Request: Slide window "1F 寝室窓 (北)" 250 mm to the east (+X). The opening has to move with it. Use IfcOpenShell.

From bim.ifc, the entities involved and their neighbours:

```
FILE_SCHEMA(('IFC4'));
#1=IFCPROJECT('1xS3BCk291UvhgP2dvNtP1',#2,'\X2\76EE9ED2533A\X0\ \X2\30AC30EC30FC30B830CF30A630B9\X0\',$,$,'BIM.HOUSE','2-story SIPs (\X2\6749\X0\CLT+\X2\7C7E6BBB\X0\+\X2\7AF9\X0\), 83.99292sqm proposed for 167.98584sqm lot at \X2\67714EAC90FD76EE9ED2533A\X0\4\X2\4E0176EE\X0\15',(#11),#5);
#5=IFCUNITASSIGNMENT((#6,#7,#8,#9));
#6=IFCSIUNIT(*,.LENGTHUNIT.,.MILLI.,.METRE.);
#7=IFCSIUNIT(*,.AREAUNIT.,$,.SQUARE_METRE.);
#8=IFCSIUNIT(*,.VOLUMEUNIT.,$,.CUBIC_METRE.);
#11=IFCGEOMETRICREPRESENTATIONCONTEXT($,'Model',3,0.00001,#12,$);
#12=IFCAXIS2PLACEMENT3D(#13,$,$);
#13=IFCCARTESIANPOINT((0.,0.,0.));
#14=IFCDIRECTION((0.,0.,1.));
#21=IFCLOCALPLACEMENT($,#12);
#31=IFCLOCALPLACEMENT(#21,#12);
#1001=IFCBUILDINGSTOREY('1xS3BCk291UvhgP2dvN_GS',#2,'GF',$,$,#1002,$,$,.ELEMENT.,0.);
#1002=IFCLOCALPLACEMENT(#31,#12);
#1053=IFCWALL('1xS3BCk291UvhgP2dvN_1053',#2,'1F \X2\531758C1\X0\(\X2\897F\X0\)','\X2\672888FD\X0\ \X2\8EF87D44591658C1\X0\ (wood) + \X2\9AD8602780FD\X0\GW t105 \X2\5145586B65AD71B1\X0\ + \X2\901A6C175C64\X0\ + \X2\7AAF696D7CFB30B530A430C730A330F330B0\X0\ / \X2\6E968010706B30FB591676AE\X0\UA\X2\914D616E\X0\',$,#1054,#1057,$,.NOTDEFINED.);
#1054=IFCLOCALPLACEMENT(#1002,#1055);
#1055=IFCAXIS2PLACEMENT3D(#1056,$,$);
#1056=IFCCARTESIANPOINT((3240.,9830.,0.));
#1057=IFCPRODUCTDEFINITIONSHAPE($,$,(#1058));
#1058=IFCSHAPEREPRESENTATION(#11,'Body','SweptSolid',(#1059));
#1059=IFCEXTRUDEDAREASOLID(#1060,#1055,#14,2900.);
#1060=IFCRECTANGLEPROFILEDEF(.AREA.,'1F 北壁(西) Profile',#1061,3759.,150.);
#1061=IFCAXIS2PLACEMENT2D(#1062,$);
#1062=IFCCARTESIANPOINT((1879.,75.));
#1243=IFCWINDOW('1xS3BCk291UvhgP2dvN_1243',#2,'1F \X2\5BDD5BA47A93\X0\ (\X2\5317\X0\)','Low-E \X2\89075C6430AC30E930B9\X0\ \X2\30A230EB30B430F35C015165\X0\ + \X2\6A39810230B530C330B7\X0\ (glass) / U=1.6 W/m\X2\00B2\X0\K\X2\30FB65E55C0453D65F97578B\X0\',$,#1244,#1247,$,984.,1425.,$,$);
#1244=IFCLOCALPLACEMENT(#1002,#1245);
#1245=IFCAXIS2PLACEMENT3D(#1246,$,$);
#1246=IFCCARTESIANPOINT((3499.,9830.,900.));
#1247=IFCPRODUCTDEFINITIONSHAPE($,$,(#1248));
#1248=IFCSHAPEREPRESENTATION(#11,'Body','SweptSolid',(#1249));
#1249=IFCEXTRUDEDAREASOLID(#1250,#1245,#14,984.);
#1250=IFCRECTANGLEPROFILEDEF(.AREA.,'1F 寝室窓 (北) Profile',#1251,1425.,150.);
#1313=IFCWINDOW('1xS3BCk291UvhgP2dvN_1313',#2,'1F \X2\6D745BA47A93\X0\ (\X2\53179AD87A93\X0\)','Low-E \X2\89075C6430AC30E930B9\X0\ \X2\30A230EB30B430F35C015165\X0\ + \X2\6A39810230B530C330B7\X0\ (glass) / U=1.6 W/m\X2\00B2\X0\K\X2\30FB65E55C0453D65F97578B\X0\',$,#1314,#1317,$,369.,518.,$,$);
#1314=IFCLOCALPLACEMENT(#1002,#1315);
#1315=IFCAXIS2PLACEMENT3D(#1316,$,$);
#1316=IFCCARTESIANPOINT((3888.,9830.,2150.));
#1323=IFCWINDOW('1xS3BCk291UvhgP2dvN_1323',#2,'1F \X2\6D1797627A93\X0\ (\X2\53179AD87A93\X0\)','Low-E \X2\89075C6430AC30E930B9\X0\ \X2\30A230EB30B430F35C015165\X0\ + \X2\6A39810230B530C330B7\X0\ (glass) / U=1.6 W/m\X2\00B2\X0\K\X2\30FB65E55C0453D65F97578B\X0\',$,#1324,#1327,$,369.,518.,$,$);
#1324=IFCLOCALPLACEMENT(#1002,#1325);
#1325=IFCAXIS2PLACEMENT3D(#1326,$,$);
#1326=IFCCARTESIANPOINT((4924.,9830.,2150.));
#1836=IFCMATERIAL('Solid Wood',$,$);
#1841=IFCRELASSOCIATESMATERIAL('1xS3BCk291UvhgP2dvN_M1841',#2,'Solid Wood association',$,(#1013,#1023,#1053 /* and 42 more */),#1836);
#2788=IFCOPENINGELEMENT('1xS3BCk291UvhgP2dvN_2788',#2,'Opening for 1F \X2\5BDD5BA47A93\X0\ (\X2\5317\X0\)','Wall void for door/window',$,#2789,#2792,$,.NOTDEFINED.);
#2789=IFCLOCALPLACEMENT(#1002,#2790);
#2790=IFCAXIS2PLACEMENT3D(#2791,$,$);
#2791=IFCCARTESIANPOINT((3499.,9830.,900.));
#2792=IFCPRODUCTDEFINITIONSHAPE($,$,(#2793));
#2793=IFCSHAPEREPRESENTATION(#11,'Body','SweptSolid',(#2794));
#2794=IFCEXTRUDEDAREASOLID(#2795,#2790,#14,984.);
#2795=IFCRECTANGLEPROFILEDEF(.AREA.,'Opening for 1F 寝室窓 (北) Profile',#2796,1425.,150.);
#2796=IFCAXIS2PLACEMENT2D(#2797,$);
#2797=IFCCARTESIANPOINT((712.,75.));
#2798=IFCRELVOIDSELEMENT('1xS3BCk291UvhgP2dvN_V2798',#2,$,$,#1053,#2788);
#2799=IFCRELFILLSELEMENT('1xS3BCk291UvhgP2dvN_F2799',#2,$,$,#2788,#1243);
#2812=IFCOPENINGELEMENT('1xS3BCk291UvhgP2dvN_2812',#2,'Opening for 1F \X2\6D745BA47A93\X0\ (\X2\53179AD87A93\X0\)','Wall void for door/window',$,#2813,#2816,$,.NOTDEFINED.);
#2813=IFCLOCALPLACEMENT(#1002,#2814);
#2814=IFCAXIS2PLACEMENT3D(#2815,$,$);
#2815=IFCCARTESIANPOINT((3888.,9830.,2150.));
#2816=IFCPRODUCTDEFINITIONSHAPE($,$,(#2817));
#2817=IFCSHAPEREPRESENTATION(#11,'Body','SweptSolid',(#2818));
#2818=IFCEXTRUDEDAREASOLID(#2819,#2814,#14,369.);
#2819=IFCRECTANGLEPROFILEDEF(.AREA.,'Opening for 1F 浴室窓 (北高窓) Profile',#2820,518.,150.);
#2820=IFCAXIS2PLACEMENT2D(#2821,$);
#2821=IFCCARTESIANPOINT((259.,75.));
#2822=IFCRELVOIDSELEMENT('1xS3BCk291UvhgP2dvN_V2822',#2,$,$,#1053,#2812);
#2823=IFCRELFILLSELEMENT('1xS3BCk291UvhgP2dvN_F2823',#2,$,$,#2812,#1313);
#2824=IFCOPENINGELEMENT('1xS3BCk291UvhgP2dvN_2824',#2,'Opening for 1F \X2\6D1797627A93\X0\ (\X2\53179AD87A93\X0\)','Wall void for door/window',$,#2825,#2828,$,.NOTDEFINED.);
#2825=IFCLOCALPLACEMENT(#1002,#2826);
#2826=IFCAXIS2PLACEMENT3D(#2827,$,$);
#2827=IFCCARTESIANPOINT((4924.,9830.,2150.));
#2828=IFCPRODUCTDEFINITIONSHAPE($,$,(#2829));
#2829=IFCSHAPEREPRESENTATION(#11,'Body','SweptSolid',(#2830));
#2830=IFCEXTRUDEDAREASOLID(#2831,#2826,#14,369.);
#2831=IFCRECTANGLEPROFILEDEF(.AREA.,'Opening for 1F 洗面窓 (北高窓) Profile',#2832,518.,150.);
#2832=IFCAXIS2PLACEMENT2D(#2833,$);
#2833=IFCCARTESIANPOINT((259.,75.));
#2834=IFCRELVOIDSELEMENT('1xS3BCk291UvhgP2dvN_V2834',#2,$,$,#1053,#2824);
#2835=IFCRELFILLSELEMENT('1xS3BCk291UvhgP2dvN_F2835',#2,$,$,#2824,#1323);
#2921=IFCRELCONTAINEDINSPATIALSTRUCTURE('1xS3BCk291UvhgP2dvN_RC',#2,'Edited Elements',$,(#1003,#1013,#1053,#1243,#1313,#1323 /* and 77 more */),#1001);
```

```python
import ifcopenshell
import ifcopenshell.api.geometry
import ifcopenshell.util.placement

model = ifcopenshell.open("bim.ifc")

window = model.by_id(1243)
opening = window.FillsVoids[0].RelatingOpeningElement
wall = opening.VoidsElements[0].RelatingBuildingElement

wall_matrix = ifcopenshell.util.placement.get_local_placement(wall.ObjectPlacement)
shift = wall_matrix[:3, 0] * 250.0
before = ifcopenshell.util.placement.get_local_placement(window.ObjectPlacement)[:3, 3].copy()

# The window is not placed relative to its opening, so move both.
for product in (opening, window):
    matrix = ifcopenshell.util.placement.get_local_placement(product.ObjectPlacement)
    matrix[:3, 3] += shift
    ifcopenshell.api.geometry.edit_object_placement(model, product=product, matrix=matrix, is_si=False)

after = ifcopenshell.util.placement.get_local_placement(window.ObjectPlacement)[:3, 3]
print("window moved by", (after - before).round(3) + 0.0)

model.write("bim_v2.ifc")
```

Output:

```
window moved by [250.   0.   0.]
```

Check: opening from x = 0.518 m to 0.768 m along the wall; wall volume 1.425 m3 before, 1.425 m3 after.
